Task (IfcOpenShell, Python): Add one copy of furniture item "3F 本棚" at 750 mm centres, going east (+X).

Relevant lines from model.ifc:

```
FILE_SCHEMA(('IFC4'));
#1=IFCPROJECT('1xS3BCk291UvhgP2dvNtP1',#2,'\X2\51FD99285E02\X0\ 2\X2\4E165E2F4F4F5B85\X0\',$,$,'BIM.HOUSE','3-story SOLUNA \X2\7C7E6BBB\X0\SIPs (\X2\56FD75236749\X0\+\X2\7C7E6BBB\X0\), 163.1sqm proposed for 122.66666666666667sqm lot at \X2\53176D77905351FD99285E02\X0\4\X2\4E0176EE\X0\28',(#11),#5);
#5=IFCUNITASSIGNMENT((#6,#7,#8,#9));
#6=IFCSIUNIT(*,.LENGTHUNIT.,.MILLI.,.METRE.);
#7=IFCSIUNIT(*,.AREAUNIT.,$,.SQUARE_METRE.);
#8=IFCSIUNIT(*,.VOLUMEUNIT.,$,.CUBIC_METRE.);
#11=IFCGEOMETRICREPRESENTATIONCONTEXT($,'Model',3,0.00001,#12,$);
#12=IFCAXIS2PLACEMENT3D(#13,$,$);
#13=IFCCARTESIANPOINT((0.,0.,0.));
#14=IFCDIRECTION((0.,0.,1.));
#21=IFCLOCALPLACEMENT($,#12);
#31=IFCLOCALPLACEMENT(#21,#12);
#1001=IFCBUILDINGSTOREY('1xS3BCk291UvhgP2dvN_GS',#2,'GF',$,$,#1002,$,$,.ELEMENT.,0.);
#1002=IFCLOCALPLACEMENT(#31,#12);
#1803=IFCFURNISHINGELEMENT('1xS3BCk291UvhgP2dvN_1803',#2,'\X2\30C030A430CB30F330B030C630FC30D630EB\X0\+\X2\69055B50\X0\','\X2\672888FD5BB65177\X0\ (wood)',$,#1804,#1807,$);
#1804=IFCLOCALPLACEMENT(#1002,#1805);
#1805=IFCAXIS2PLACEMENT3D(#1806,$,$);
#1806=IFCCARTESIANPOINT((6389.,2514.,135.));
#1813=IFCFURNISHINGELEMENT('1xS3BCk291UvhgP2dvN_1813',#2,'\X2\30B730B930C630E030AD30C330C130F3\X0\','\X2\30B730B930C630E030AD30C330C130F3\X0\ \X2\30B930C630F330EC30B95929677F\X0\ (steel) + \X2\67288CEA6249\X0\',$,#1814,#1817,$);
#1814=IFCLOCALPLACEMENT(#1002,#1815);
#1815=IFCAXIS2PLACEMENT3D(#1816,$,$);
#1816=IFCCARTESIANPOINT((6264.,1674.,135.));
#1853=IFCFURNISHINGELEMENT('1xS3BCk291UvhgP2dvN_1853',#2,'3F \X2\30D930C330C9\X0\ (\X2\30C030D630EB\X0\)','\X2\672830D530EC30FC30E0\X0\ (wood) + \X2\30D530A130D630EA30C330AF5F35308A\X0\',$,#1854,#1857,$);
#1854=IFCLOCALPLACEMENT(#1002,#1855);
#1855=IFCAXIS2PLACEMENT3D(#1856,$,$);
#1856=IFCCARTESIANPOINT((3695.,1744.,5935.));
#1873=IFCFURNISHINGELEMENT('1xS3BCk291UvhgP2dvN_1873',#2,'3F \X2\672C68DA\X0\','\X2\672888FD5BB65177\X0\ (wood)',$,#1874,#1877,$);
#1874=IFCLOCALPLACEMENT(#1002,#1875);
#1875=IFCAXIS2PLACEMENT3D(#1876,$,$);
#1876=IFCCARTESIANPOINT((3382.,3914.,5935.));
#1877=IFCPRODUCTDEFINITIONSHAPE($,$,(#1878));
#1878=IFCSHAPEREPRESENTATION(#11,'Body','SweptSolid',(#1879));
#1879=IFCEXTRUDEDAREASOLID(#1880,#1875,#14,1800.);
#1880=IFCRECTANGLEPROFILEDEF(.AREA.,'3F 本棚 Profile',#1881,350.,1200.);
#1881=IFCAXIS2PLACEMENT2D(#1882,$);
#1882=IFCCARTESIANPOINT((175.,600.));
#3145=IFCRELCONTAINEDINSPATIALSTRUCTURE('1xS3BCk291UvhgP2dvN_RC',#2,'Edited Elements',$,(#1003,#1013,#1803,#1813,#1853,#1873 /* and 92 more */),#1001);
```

```python
import numpy as np
import ifcopenshell
import ifcopenshell.api.geometry
import ifcopenshell.api.root
import ifcopenshell.util.element
import ifcopenshell.util.placement
import ifcopenshell.util.unit

model = ifcopenshell.open("model.ifc")
unit_scale = ifcopenshell.util.unit.calculate_unit_scale(model)


def reuse_history(source, copy):
    """copy_class also copies each property set's owner history, people and application; keep the originals."""
    for rel in copy.IsDefinedBy:
        if rel.is_a("IfcRelDefinesByProperties") and (history := rel.RelatingPropertyDefinition.OwnerHistory):
            rel.RelatingPropertyDefinition.OwnerHistory = source.OwnerHistory
            ifcopenshell.util.element.remove_deep2(model, history)


source = model.by_id(1873)
base = ifcopenshell.util.placement.get_local_placement(source.ObjectPlacement)
step = np.array([1.0, 0.0, 0.0]) * 0.75 / unit_scale

for i in range(1, 2):
    copy = ifcopenshell.api.root.copy_class(model, product=source)
    copy.Representation = ifcopenshell.util.element.copy_deep(
        model, source.Representation, exclude=["IfcGeometricRepresentationContext", "IfcRepresentationMap"]
    )
    reuse_history(source, copy)
    matrix = base.copy()
    matrix[:3, 3] += i * step
    print("added at", matrix[:3, 3].round(3) + 0.0)
    ifcopenshell.api.geometry.edit_object_placement(model, product=copy, matrix=matrix, is_si=False)

model.write("model_updated.ifc")
```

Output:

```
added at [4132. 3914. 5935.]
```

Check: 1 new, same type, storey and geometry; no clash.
